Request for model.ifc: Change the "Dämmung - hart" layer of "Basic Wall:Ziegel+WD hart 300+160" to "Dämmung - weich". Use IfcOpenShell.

First a look at what the model holds.

```python
import ifcopenshell
import ifcopenshell.util.element

model = ifcopenshell.open("model.ifc")
print(model.schema)
for layer_set in model.by_type("IfcMaterialLayerSet"):
    if layer_set.LayerSetName == "Basic Wall:Ziegel+WD hart 300+160":
        for layer in layer_set.MaterialLayers:
            print(layer.id(), layer.Material and layer.Material.Name, layer.LayerThickness, sep=" | ")
        print(len(ifcopenshell.util.element.get_elements_by_material(model, layer_set)), "elements and types use it")
print(sorted(m.Name for m in model.by_type("IfcMaterial") if m.Name)[:60])
```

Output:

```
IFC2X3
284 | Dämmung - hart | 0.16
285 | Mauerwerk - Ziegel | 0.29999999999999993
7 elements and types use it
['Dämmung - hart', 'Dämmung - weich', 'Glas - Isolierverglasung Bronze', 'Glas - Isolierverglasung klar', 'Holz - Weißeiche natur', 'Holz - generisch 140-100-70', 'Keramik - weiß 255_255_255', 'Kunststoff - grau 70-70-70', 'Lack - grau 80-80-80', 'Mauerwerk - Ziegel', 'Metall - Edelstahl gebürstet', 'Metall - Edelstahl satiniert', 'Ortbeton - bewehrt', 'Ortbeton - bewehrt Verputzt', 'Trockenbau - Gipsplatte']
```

```python
import ifcopenshell
import ifcopenshell.api.material

model = ifcopenshell.open("model.ifc")

layer_set = next(s for s in model.by_type("IfcMaterialLayerSet") if s.LayerSetName == "Basic Wall:Ziegel+WD hart 300+160")
layer = next(l for l in layer_set.MaterialLayers if l.Material and l.Material.Name == "Dämmung - hart")
material = next(m for m in model.by_type("IfcMaterial") if m.Name == "Dämmung - weich")

# Point this one layer at the other material; renaming the old one would change it everywhere.
ifcopenshell.api.material.edit_layer(model, layer=layer, attributes={}, material=material)

print([l.Material.Name if l.Material else None for l in layer_set.MaterialLayers])

model.write("model_v2.ifc")
```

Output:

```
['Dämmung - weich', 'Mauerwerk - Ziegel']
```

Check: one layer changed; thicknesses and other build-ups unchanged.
